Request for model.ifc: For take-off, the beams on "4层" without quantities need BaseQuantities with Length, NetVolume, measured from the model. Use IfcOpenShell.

First a look at what the model holds.

```python
import ifcopenshell
import ifcopenshell.util.element
import ifcopenshell.util.unit

model = ifcopenshell.open("model.ifc")
print(model.schema)
for unit_type in ("LENGTHUNIT", "AREAUNIT", "VOLUMEUNIT"):
    print(unit_type, ifcopenshell.util.unit.calculate_unit_scale(model, unit_type))
storey = next(s for s in model.by_type("IfcBuildingStorey") if s.Name == "4层")
beams = [e for e in ifcopenshell.util.element.get_decomposition(storey) if e.is_a("IfcBeam")]
for e in sorted(beams, key=lambda e: e.id()):
    print(e.id(), e.is_a(), e.Name, list(ifcopenshell.util.element.get_psets(e, qtos_only=True)), sep=" | ")
```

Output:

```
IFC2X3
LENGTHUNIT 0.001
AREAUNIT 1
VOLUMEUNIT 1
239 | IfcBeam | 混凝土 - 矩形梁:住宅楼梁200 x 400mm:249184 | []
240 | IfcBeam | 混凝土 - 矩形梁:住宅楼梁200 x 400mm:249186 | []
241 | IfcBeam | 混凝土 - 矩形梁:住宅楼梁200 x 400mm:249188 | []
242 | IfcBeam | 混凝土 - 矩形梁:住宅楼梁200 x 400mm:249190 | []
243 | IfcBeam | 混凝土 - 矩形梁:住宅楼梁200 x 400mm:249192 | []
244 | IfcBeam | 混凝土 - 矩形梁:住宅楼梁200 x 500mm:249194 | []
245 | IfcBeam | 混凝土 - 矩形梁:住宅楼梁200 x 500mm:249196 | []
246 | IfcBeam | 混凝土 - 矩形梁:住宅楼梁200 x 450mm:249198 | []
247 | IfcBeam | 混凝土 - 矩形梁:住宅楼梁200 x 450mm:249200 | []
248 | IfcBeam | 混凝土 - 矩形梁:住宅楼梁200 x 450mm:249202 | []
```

```python
import ifcopenshell
import ifcopenshell.api.pset
import ifcopenshell.geom
import ifcopenshell.util.element
import ifcopenshell.util.shape
import ifcopenshell.util.unit

model = ifcopenshell.open("model.ifc")
unit_scale = ifcopenshell.util.unit.calculate_unit_scale(model)
volume_scale = ifcopenshell.util.unit.calculate_unit_scale(model, "VOLUMEUNIT")
settings = ifcopenshell.geom.settings()

storey = next(s for s in model.by_type("IfcBuildingStorey") if s.Name == "4层")
beams = [e for e in ifcopenshell.util.element.get_decomposition(storey) if e.is_a("IfcBeam")]

for e in sorted(beams, key=lambda e: e.id()):
    if ifcopenshell.util.element.get_psets(e, qtos_only=True, should_inherit=False):
        continue
    # Geometry comes back in metres, in the element's own axes.
    shape = ifcopenshell.geom.create_shape(settings, e)
    values = {
        "Length": ifcopenshell.util.shape.get_max_xyz(shape.geometry) / unit_scale,
        "NetVolume": ifcopenshell.util.shape.get_volume(shape.geometry) / volume_scale,
    }
    qto = ifcopenshell.api.pset.add_qto(model, product=e, name="BaseQuantities")
    ifcopenshell.api.pset.edit_qto(model, qto=qto, properties=values)
    print(e.id(), {k: round(v, 3) for k, v in values.items()})

model.write("model_v2.ifc")
```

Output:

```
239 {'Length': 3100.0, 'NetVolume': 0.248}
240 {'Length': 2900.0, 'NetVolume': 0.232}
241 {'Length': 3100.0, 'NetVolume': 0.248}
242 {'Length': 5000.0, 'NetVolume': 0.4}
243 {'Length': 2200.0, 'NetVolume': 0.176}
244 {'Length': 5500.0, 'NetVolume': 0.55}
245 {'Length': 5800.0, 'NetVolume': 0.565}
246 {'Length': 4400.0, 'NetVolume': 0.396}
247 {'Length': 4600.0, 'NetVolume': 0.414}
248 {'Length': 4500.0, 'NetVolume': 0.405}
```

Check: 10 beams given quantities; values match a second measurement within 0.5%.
